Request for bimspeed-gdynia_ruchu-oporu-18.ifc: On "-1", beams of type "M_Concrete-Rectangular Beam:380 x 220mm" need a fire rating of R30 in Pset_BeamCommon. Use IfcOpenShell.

First a look at what the model holds.

```python
import ifcopenshell
import ifcopenshell.util.element

model = ifcopenshell.open("bimspeed-gdynia_ruchu-oporu-18.ifc")
print(model.schema)
storey = next(s for s in model.by_type("IfcBuildingStorey") if s.Name == "-1")
beams = [e for e in ifcopenshell.util.element.get_decomposition(storey) if e.is_a("IfcBeam")]
seen = {}
for e in beams:
    element_type = ifcopenshell.util.element.get_type(e)
    key = (element_type.Name if element_type != e and element_type else None, ifcopenshell.util.element.get_pset(e, "Pset_BeamCommon", "FireRating"))
    seen[key] = seen.get(key, 0) + 1
for (name, value), count in sorted(seen.items(), key=str):
    print(count, "x", name, "|", value)
```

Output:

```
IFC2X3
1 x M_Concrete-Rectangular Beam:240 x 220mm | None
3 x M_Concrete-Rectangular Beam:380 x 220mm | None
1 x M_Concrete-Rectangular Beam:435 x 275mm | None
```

```python
import ifcopenshell
import ifcopenshell.api.pset
import ifcopenshell.util.element

model = ifcopenshell.open("bimspeed-gdynia_ruchu-oporu-18.ifc")

storey = next(s for s in model.by_type("IfcBuildingStorey") if s.Name == "-1")
beams = [e for e in ifcopenshell.util.element.get_decomposition(storey) if e.is_a("IfcBeam")]

count = 0
for e in beams:
    element_type = ifcopenshell.util.element.get_type(e)
    if element_type in (None, e) or element_type.Name != "M_Concrete-Rectangular Beam:380 x 220mm":
        continue
    # add_pset returns the element's existing set when there is one.
    pset = ifcopenshell.api.pset.add_pset(model, product=e, name="Pset_BeamCommon")
    ifcopenshell.api.pset.edit_pset(model, pset=pset, properties={"FireRating": "R30"})
    count += 1

print(count, "beams updated")

model.write("bimspeed-gdynia_ruchu-oporu-18_updated.ifc")
```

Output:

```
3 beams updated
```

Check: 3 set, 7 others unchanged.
